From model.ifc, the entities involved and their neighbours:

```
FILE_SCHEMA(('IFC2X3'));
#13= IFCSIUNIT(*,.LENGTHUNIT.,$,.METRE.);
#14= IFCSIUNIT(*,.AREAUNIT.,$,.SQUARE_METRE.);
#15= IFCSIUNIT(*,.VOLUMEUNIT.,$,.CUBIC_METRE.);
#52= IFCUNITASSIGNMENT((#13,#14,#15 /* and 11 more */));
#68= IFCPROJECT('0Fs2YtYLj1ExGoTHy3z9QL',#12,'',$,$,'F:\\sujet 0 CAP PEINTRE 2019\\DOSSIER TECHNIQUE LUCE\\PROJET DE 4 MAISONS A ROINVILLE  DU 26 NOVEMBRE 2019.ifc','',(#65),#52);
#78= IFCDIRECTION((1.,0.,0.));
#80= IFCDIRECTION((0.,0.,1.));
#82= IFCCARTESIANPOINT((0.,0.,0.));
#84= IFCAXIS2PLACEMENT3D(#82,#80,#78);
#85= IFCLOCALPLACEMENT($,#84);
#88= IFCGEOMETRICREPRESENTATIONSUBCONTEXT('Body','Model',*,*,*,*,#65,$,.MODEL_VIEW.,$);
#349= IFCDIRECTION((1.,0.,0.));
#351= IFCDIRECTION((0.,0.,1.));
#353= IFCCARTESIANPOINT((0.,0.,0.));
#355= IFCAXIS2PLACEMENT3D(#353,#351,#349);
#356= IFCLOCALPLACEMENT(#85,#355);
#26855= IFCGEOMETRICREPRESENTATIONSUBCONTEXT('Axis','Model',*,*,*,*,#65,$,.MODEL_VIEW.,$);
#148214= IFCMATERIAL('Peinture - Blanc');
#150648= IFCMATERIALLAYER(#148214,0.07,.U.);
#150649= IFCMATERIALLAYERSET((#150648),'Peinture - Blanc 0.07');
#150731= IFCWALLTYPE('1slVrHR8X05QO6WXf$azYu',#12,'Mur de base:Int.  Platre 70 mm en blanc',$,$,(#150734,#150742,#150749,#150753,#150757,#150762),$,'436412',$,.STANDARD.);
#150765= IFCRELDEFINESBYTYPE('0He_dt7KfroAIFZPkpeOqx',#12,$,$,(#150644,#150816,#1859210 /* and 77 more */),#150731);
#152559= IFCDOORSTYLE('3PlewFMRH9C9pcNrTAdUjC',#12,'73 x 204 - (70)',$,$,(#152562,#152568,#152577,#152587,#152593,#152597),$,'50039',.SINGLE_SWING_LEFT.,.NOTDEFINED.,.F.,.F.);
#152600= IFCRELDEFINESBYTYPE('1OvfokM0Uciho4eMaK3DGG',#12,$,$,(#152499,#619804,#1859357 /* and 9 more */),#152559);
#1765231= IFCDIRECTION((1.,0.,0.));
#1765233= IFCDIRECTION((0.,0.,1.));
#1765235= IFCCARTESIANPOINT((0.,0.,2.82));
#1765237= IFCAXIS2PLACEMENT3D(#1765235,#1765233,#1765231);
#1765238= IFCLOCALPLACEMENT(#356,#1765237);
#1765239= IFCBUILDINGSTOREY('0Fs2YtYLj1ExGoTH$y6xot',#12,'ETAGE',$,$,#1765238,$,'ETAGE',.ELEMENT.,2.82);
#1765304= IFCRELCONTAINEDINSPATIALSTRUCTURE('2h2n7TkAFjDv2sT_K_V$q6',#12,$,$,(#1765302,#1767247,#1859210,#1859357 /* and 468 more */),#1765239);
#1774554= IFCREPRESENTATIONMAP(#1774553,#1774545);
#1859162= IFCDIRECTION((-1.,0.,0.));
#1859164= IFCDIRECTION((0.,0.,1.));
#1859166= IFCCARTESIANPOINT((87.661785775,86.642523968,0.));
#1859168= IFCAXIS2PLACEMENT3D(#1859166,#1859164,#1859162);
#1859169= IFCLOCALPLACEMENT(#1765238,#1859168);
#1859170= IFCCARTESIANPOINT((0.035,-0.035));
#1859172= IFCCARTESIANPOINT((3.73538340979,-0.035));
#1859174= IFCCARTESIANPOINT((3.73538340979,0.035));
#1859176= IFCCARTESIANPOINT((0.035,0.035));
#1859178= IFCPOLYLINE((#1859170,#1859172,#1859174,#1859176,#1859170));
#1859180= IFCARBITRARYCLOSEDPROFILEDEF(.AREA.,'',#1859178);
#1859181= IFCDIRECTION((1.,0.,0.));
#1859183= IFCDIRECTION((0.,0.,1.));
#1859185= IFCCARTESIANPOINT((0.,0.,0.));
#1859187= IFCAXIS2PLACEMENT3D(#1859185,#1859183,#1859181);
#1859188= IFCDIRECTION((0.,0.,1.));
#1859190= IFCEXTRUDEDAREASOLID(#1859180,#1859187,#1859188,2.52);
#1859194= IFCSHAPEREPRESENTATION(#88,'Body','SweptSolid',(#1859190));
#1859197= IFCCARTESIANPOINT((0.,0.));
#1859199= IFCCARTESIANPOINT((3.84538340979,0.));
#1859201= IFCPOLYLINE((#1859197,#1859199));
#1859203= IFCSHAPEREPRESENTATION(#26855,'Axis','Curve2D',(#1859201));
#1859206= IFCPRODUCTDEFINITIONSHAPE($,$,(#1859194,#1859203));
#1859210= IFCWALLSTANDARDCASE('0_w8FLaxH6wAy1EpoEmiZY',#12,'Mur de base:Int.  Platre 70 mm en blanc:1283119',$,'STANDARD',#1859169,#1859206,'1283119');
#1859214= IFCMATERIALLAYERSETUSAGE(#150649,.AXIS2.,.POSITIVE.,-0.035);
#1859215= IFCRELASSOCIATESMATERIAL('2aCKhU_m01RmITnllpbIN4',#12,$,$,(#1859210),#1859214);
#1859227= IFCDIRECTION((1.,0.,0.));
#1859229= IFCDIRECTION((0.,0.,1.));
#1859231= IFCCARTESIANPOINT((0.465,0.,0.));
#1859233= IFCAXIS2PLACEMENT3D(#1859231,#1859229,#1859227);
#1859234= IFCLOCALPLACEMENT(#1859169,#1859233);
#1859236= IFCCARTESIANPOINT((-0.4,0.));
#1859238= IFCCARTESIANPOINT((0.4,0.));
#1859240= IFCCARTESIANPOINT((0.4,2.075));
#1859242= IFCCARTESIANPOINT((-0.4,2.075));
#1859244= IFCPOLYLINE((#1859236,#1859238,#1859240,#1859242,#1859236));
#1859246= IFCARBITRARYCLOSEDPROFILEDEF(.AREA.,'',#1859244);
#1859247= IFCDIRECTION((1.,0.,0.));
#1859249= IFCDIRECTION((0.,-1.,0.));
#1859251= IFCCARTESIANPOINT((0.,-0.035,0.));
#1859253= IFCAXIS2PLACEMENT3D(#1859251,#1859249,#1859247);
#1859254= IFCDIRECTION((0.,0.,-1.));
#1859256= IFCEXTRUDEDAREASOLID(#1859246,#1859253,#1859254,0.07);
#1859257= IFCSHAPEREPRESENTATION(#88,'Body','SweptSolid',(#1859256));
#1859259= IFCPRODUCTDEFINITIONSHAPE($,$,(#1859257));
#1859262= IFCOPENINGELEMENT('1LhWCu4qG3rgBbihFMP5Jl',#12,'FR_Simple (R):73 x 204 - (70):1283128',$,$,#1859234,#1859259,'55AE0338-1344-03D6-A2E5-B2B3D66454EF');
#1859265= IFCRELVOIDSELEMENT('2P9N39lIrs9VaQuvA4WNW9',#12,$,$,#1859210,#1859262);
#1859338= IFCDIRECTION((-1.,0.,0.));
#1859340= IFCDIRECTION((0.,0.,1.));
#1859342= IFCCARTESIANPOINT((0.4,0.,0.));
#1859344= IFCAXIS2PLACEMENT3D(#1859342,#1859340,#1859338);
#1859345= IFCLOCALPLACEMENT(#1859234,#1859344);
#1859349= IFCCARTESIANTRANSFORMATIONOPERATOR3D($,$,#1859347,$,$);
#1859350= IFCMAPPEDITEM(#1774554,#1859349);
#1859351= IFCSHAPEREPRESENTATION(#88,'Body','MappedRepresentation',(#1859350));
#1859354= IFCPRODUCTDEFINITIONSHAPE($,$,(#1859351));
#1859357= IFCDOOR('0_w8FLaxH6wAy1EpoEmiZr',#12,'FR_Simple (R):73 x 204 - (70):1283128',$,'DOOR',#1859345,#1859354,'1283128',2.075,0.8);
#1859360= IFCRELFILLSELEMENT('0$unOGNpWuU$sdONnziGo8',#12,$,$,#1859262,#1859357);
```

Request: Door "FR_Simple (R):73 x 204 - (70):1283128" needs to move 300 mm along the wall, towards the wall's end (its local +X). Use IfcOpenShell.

```python
import ifcopenshell
import ifcopenshell.api.geometry
import ifcopenshell.util.placement

model = ifcopenshell.open("model.ifc")

door = model.by_guid("0_w8FLaxH6wAy1EpoEmiZr")
opening = door.FillsVoids[0].RelatingOpeningElement
wall = opening.VoidsElements[0].RelatingBuildingElement

wall_matrix = ifcopenshell.util.placement.get_local_placement(wall.ObjectPlacement)
shift = wall_matrix[:3, 0] * 0.3
before = ifcopenshell.util.placement.get_local_placement(door.ObjectPlacement)[:3, 3].copy()

# The door is placed relative to its opening, so it follows when the opening moves.
matrix = ifcopenshell.util.placement.get_local_placement(opening.ObjectPlacement)
matrix[:3, 3] += shift
ifcopenshell.api.geometry.edit_object_placement(
    model, product=opening, matrix=matrix, is_si=False, should_transform_children=True
)

after = ifcopenshell.util.placement.get_local_placement(door.ObjectPlacement)[:3, 3]
print("door moved by", (after - before).round(3) + 0.0)

model.write("model_edited.ifc")
```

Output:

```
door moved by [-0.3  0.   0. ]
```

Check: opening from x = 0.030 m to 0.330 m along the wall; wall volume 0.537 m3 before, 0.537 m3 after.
